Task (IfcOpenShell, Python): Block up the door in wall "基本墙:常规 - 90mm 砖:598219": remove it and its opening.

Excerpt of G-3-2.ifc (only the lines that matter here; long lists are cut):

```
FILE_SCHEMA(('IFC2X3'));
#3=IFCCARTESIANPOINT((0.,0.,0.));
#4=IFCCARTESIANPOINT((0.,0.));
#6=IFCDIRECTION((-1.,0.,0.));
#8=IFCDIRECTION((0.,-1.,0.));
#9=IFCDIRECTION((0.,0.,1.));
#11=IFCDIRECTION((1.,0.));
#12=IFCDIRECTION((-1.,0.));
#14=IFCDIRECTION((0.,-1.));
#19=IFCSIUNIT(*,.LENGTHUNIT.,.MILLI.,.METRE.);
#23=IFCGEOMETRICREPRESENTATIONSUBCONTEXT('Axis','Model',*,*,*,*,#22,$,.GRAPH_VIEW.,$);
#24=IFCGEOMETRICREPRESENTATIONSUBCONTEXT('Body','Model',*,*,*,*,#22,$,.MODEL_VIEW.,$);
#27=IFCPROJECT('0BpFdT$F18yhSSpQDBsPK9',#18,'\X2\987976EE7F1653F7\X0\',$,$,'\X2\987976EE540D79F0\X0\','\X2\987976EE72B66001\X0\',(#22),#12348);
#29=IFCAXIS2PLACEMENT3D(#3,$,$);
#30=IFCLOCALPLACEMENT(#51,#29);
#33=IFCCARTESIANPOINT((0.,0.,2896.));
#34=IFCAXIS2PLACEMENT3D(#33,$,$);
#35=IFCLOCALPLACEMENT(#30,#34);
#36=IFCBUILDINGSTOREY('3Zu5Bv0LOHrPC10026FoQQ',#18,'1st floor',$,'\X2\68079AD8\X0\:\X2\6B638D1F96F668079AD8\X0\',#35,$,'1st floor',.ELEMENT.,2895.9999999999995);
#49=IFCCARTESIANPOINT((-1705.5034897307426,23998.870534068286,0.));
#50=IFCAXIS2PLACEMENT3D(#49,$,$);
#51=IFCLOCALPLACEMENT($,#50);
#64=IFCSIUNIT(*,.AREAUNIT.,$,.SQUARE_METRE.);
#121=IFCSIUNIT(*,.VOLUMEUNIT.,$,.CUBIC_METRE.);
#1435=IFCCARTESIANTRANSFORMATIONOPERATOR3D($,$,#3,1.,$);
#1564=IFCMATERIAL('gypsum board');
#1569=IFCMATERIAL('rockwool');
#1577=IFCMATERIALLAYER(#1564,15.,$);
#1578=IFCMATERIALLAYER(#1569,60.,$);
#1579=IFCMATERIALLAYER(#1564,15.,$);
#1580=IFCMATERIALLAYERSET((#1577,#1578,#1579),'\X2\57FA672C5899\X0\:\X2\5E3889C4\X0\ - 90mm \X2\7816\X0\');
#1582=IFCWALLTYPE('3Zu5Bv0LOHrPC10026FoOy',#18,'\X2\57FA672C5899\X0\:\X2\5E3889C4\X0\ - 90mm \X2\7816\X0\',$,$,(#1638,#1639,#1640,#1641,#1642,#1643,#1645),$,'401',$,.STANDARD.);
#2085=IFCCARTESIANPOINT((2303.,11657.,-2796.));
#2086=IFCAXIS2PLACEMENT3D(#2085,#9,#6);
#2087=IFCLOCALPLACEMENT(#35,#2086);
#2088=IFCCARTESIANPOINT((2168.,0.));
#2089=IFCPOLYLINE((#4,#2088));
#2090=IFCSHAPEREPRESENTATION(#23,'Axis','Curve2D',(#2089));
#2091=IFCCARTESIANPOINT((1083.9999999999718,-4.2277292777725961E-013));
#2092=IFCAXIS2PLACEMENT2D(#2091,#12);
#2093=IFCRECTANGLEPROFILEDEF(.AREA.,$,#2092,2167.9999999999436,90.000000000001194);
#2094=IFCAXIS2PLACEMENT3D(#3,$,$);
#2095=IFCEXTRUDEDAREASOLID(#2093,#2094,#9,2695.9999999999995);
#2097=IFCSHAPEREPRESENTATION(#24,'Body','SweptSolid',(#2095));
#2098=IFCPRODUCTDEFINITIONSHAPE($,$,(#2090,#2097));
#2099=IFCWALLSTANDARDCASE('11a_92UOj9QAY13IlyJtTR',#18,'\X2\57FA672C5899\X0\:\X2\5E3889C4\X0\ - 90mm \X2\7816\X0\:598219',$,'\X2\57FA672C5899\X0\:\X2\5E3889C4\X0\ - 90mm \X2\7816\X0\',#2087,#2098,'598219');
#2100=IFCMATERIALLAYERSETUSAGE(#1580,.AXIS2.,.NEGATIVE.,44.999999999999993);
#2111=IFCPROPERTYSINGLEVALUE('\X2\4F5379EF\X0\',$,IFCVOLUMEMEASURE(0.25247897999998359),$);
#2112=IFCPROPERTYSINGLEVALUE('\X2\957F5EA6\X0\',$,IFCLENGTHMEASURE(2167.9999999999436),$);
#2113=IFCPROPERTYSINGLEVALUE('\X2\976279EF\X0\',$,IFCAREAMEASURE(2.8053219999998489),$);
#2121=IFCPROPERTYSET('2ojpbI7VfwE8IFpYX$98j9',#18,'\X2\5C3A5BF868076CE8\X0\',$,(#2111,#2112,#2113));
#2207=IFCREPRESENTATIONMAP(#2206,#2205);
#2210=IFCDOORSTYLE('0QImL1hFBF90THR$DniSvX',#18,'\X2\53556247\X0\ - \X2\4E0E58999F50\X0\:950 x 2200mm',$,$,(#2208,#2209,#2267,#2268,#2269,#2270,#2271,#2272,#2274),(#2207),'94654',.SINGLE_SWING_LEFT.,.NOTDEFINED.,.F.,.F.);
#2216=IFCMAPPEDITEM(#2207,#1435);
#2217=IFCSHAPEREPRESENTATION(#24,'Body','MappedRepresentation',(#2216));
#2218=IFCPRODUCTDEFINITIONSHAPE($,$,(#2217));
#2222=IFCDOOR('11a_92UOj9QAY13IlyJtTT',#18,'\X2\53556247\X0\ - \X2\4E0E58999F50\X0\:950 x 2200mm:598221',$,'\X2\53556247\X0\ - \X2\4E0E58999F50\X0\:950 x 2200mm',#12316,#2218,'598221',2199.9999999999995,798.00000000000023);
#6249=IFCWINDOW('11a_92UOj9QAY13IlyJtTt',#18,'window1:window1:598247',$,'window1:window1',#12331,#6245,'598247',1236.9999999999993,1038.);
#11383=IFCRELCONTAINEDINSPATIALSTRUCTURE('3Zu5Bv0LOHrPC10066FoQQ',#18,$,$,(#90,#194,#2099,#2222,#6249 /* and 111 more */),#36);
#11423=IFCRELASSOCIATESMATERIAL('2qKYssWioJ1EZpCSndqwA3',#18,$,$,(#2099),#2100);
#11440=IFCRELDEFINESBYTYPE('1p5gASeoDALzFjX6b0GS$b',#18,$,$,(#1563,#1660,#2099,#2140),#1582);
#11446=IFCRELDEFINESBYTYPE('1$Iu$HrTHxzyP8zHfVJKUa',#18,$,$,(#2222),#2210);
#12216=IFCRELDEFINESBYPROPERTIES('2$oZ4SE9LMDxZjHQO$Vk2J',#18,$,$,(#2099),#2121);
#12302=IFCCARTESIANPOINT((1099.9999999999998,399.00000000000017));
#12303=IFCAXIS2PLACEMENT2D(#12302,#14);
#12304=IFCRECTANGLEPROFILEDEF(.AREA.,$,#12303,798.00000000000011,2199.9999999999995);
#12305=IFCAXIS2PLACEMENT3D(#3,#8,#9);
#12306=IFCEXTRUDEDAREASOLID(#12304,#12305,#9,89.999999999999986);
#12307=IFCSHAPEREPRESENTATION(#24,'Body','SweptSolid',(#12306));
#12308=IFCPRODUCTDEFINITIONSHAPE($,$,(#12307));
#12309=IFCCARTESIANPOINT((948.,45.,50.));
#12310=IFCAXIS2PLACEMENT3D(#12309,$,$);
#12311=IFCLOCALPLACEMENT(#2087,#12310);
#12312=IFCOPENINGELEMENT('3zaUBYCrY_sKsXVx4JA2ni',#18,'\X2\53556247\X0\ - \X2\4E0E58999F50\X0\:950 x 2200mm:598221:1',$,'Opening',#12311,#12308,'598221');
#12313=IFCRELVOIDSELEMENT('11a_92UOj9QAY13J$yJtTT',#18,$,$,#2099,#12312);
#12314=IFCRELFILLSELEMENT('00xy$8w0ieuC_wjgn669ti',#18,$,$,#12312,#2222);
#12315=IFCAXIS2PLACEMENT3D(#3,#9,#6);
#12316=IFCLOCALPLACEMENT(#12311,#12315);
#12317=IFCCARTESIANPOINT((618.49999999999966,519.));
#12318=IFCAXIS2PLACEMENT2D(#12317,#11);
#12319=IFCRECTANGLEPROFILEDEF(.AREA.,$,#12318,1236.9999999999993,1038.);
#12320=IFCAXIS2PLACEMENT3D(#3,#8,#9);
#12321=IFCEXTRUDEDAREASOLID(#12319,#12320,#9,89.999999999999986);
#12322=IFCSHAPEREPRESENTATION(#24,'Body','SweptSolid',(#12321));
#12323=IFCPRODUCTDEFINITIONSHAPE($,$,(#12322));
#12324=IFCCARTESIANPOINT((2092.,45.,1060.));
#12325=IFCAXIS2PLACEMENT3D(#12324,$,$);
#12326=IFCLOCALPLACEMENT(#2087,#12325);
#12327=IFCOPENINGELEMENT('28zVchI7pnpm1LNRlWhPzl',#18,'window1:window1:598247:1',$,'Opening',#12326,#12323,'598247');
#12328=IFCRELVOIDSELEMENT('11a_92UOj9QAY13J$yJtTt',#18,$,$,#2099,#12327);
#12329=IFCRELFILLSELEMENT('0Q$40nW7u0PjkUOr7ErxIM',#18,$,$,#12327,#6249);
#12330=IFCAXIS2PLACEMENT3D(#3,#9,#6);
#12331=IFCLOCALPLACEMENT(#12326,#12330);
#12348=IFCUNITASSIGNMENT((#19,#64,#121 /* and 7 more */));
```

```python
import ifcopenshell
import ifcopenshell.api.feature
import ifcopenshell.api.pset
import ifcopenshell.api.root
import ifcopenshell.geom
import ifcopenshell.util.element
import ifcopenshell.util.shape
import ifcopenshell.util.unit

model = ifcopenshell.open("G-3-2.ifc")
area_scale = ifcopenshell.util.unit.calculate_unit_scale(model, "AREAUNIT")
volume_scale = ifcopenshell.util.unit.calculate_unit_scale(model, "VOLUMEUNIT")
settings = ifcopenshell.geom.settings()


def volume(element):
    """Net volume in cubic metres, openings subtracted."""
    shape = ifcopenshell.geom.create_shape(settings, element)
    return ifcopenshell.util.shape.get_volume(shape.geometry)


door = model.by_guid("11a_92UOj9QAY13IlyJtTT")
opening = door.FillsVoids[0].RelatingOpeningElement
wall = opening.VoidsElements[0].RelatingBuildingElement
before = volume(wall)

ifcopenshell.api.root.remove_product(model, product=door)
ifcopenshell.api.feature.remove_feature(model, feature=opening)

after = volume(wall)
thickness = 0.09  # wall thickness in metres

# Update the wall's stored quantities.
pset = model.by_id(ifcopenshell.util.element.get_pset(wall, "尺寸标注", should_inherit=False)["id"])
ifcopenshell.api.pset.edit_pset(model, pset=pset, properties={
    "体积": model.create_entity("IfcVolumeMeasure", after / volume_scale),
    "面积": model.create_entity("IfcAreaMeasure", after / thickness / area_scale),
})

print(f"wall volume {before:.3f} -> {after:.3f} m3")

model.write("G-3-2-out.ifc")
```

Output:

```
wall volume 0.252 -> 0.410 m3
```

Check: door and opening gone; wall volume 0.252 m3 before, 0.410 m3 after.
